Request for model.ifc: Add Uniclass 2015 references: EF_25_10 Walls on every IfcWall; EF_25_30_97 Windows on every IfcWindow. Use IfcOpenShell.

First a look at what the model holds.

```python
import ifcopenshell

model = ifcopenshell.open("model.ifc")
print(model.schema)
print("classifications:", [c.Name for c in model.by_type("IfcClassification")])
for ifc_class in ("IfcDoor", "IfcRoof", "IfcStair", "IfcWall", "IfcWindow"):
    print(ifc_class, len(model.by_type(ifc_class)))
```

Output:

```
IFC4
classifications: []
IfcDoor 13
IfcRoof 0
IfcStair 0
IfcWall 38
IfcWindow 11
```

```python
import ifcopenshell
import ifcopenshell.api.classification

model = ifcopenshell.open("model.ifc")

system = ifcopenshell.api.classification.add_classification(model, classification="Uniclass 2015")

codes = {
    "IfcWall": ("EF_25_10", "Walls"),
    "IfcWindow": ("EF_25_30_97", "Windows"),
}
for ifc_class, (code, name) in codes.items():
    products = model.by_type(ifc_class)
    ifcopenshell.api.classification.add_reference(
        model, products=products, classification=system, identification=code, name=name
    )
    print(code, len(products))

model.write("model_updated.ifc")
```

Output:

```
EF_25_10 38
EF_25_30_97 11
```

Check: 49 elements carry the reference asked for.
